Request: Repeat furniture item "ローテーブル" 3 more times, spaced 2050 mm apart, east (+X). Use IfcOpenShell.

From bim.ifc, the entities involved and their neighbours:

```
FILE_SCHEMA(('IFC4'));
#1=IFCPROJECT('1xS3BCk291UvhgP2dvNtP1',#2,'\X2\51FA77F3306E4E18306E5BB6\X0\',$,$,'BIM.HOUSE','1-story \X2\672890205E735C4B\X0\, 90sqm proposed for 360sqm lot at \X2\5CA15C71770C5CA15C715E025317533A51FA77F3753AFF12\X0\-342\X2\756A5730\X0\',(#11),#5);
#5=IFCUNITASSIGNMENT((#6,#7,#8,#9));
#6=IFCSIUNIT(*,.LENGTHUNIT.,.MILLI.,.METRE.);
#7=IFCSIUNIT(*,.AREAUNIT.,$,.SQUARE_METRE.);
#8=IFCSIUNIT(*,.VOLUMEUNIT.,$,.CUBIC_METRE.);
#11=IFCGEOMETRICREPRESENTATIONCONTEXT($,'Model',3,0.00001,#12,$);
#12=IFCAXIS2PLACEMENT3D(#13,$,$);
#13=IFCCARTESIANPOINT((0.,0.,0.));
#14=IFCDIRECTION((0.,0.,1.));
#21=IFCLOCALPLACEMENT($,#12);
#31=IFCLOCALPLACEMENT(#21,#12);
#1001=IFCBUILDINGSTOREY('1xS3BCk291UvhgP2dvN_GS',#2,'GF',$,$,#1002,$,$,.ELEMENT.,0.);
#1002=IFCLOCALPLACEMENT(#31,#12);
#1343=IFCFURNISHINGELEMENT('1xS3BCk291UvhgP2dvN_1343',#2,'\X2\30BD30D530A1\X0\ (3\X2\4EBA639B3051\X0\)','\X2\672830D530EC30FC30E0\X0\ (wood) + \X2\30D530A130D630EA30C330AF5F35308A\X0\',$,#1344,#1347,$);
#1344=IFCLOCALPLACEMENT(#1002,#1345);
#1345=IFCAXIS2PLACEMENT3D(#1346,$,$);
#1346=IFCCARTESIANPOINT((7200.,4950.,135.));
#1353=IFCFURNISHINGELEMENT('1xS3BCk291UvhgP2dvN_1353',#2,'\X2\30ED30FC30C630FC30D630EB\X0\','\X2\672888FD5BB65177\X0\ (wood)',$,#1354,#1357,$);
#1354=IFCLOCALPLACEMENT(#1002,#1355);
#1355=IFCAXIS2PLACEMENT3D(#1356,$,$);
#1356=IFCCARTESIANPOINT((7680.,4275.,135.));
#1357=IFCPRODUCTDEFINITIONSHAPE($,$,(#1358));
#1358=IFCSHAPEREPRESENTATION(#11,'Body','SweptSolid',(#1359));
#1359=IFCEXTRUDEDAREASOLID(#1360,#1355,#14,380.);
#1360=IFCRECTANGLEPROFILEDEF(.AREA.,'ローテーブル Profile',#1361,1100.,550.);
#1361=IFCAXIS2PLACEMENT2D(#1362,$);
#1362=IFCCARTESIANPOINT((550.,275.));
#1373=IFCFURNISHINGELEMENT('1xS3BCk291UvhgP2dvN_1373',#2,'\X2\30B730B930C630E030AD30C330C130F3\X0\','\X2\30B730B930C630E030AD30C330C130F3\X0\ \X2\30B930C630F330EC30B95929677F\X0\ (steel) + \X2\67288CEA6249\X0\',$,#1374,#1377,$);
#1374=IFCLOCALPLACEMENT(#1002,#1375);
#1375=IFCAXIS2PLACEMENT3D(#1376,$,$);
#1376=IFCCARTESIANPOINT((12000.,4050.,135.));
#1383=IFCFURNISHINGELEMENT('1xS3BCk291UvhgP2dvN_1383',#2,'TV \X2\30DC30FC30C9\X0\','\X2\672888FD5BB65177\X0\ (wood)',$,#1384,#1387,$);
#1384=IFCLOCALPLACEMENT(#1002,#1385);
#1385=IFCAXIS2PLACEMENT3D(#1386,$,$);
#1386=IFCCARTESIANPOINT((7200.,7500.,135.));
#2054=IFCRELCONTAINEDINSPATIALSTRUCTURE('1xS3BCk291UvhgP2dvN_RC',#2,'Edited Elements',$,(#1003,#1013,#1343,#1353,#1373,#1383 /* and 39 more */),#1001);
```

```python
import numpy as np
import ifcopenshell
import ifcopenshell.api.geometry
import ifcopenshell.api.root
import ifcopenshell.util.element
import ifcopenshell.util.placement
import ifcopenshell.util.unit

model = ifcopenshell.open("bim.ifc")
unit_scale = ifcopenshell.util.unit.calculate_unit_scale(model)


def reuse_history(source, copy):
    """copy_class also copies each property set's owner history, people and application; keep the originals."""
    for rel in copy.IsDefinedBy:
        if rel.is_a("IfcRelDefinesByProperties") and (history := rel.RelatingPropertyDefinition.OwnerHistory):
            rel.RelatingPropertyDefinition.OwnerHistory = source.OwnerHistory
            ifcopenshell.util.element.remove_deep2(model, history)


source = model.by_id(1353)
base = ifcopenshell.util.placement.get_local_placement(source.ObjectPlacement)
step = np.array([1.0, 0.0, 0.0]) * 2.05 / unit_scale

for i in range(1, 4):
    copy = ifcopenshell.api.root.copy_class(model, product=source)
    copy.Representation = ifcopenshell.util.element.copy_deep(
        model, source.Representation, exclude=["IfcGeometricRepresentationContext", "IfcRepresentationMap"]
    )
    reuse_history(source, copy)
    matrix = base.copy()
    matrix[:3, 3] += i * step
    print("added at", matrix[:3, 3].round(3) + 0.0)
    ifcopenshell.api.geometry.edit_object_placement(model, product=copy, matrix=matrix, is_si=False)

model.write("bim_v2.ifc")
```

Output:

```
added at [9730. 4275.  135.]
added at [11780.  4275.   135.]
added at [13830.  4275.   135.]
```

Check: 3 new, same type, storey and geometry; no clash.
